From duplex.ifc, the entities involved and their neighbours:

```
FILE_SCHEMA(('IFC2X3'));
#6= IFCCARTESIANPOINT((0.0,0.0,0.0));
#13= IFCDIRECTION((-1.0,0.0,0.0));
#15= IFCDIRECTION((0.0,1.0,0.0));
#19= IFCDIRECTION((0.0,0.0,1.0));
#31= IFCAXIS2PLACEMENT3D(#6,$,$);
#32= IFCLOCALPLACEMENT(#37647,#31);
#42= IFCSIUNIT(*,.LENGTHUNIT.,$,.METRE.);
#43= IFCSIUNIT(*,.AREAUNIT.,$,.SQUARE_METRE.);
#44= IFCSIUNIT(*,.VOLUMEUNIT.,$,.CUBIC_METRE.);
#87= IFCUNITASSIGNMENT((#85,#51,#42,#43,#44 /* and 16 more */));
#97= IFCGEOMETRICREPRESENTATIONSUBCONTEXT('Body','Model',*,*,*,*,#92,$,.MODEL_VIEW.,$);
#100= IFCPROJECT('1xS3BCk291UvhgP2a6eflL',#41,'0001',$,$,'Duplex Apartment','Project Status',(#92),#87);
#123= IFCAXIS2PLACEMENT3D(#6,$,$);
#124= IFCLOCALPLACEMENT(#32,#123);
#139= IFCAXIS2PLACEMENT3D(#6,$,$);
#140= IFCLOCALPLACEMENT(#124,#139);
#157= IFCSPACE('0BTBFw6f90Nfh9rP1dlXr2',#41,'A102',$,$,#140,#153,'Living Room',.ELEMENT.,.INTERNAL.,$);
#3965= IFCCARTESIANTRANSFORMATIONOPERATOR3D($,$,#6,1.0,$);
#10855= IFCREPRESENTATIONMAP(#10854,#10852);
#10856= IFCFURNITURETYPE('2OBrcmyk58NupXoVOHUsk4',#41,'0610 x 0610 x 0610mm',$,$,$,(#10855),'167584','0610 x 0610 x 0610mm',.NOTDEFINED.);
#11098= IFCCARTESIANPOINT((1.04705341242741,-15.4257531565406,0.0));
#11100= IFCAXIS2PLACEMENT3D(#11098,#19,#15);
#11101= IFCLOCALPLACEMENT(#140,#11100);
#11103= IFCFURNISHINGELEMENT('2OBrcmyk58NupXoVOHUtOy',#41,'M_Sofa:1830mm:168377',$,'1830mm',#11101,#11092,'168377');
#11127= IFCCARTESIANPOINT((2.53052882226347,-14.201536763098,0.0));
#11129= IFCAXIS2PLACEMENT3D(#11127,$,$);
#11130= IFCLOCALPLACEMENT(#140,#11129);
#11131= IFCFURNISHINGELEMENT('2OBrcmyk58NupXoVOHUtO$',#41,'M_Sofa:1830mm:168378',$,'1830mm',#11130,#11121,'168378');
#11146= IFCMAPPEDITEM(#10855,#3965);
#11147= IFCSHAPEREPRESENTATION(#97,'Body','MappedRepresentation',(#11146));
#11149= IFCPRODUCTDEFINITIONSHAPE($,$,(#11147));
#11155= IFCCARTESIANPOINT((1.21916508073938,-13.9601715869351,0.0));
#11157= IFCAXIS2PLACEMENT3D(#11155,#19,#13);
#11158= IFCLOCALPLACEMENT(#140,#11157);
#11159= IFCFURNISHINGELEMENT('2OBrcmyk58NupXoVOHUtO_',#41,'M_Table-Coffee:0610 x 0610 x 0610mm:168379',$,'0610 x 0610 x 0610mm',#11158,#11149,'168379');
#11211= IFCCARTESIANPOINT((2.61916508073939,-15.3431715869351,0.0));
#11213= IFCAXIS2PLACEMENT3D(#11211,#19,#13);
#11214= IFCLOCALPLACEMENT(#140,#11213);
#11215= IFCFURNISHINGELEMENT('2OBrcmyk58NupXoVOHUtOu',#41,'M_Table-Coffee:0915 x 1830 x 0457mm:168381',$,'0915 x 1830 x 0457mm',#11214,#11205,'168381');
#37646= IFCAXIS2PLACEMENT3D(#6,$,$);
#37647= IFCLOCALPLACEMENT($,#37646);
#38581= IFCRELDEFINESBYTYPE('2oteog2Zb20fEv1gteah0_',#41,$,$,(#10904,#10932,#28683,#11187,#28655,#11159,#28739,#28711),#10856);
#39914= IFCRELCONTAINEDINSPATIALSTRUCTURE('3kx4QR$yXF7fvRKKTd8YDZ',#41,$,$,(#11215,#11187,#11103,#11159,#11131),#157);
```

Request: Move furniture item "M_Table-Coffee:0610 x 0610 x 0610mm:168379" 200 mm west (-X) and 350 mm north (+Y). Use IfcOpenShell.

```python
import ifcopenshell
import ifcopenshell.api.geometry
import ifcopenshell.util.placement
import ifcopenshell.util.unit

model = ifcopenshell.open("duplex.ifc")
unit_scale = ifcopenshell.util.unit.calculate_unit_scale(model)

item = model.by_id(11159)
matrix = ifcopenshell.util.placement.get_local_placement(item.ObjectPlacement)
matrix[0, 3] -= 0.2 / unit_scale
matrix[1, 3] += 0.35 / unit_scale
ifcopenshell.api.geometry.edit_object_placement(model, product=item, matrix=matrix, is_si=False)

print(ifcopenshell.util.placement.get_local_placement(item.ObjectPlacement).round(3) + 0.0)

model.write("duplex_edited.ifc")
```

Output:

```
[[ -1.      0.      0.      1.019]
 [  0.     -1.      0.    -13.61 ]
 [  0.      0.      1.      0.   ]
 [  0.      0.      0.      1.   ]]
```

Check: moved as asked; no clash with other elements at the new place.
